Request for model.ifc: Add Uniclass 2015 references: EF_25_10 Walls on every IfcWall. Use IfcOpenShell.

First a look at what the model holds.

```python
import ifcopenshell

model = ifcopenshell.open("model.ifc")
print(model.schema)
print("classifications:", [c.Name for c in model.by_type("IfcClassification")])
for ifc_class in ("IfcDoor", "IfcRoof", "IfcStair", "IfcWall", "IfcWindow"):
    print(ifc_class, len(model.by_type(ifc_class)))
```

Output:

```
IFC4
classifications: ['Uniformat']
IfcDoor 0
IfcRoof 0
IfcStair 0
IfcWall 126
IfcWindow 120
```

```python
import ifcopenshell
import ifcopenshell.api.classification

model = ifcopenshell.open("model.ifc")

system = ifcopenshell.api.classification.add_classification(model, classification="Uniclass 2015")

codes = {
    "IfcWall": ("EF_25_10", "Walls"),
}
for ifc_class, (code, name) in codes.items():
    products = model.by_type(ifc_class)
    ifcopenshell.api.classification.add_reference(
        model, products=products, classification=system, identification=code, name=name
    )
    print(code, len(products))

model.write("model-out.ifc")
```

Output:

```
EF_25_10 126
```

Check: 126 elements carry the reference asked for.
